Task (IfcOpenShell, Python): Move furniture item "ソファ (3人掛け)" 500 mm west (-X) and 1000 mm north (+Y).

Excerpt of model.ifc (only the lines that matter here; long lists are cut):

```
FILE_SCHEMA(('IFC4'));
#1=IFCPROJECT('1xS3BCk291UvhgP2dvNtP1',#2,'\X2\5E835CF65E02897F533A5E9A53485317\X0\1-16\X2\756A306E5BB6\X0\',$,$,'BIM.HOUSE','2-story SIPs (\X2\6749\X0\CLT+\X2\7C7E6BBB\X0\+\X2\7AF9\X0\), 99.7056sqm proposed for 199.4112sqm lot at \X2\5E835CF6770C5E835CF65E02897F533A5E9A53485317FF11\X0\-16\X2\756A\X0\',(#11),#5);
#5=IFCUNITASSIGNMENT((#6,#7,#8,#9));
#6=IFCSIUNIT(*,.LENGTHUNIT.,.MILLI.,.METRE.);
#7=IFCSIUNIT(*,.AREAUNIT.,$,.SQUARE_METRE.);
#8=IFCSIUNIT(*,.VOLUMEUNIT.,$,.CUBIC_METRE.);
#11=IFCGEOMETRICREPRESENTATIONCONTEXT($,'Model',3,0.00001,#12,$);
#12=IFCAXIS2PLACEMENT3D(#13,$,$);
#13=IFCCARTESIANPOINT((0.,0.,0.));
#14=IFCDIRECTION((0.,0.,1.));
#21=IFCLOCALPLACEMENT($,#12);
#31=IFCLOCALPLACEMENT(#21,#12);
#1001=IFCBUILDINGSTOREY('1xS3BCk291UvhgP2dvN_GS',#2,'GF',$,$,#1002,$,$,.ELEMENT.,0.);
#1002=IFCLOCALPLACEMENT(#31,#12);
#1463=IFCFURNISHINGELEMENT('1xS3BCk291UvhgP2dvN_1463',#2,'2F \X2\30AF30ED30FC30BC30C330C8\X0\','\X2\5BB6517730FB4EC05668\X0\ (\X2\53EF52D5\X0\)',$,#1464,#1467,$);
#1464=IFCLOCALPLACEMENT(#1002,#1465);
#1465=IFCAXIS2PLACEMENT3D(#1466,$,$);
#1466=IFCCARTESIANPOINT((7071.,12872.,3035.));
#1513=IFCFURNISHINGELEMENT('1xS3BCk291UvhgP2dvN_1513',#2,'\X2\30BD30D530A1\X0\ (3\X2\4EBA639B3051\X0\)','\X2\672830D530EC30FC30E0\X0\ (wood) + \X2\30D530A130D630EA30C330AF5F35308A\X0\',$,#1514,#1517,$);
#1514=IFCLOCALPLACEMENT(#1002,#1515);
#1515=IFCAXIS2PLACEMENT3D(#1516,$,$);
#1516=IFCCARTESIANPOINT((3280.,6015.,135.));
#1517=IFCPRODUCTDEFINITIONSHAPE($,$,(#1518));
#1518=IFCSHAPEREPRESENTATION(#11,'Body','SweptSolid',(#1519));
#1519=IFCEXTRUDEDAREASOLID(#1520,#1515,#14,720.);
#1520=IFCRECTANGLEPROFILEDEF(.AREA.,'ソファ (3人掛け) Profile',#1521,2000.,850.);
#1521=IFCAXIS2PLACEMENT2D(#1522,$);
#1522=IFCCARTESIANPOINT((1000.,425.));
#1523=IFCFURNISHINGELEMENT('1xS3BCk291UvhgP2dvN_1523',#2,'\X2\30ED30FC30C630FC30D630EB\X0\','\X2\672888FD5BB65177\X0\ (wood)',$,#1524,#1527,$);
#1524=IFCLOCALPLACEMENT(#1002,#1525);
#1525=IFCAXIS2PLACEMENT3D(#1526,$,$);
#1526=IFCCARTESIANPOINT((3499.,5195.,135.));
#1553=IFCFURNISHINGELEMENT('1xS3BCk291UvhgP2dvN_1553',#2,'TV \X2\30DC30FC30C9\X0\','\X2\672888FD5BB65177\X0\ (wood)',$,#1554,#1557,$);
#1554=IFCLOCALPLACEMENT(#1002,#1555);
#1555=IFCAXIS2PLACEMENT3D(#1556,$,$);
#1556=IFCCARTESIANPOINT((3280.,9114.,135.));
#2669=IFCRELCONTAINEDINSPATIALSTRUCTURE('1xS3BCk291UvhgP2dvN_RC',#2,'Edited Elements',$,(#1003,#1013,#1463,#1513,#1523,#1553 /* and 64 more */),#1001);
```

```python
import ifcopenshell
import ifcopenshell.api.geometry
import ifcopenshell.util.placement

model = ifcopenshell.open("model.ifc")

item = model.by_guid("1xS3BCk291UvhgP2dvN_1513")
matrix = ifcopenshell.util.placement.get_local_placement(item.ObjectPlacement)
matrix[0, 3] -= 500.0
matrix[1, 3] += 1000.0
ifcopenshell.api.geometry.edit_object_placement(model, product=item, matrix=matrix, is_si=False)

print(ifcopenshell.util.placement.get_local_placement(item.ObjectPlacement).round(3) + 0.0)

model.write("model_updated.ifc")
```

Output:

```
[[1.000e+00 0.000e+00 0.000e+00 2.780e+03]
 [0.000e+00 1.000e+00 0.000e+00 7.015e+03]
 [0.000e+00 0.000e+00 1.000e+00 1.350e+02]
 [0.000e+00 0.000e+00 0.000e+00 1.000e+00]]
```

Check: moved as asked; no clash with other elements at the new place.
